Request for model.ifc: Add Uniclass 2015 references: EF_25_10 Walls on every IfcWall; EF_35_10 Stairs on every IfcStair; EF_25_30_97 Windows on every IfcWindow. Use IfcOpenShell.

First a look at what the model holds.

```python
import ifcopenshell

model = ifcopenshell.open("model.ifc")
print(model.schema)
print("classifications:", [c.Name for c in model.by_type("IfcClassification")])
for ifc_class in ("IfcDoor", "IfcRoof", "IfcStair", "IfcWall", "IfcWindow"):
    print(ifc_class, len(model.by_type(ifc_class)))
```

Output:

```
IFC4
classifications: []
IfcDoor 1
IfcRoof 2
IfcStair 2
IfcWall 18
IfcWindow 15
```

```python
import ifcopenshell
import ifcopenshell.api.classification

model = ifcopenshell.open("model.ifc")

system = ifcopenshell.api.classification.add_classification(model, classification="Uniclass 2015")

codes = {
    "IfcWall": ("EF_25_10", "Walls"),
    "IfcStair": ("EF_35_10", "Stairs"),
    "IfcWindow": ("EF_25_30_97", "Windows"),
}
for ifc_class, (code, name) in codes.items():
    products = model.by_type(ifc_class)
    ifcopenshell.api.classification.add_reference(
        model, products=products, classification=system, identification=code, name=name
    )
    print(code, len(products))

model.write("model-out.ifc")
```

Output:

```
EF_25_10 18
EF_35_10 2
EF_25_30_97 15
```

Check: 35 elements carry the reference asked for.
